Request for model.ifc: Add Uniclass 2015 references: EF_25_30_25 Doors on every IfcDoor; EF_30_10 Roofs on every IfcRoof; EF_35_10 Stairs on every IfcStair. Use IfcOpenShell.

First a look at what the model holds.

```python
import ifcopenshell

model = ifcopenshell.open("model.ifc")
print(model.schema)
print("classifications:", [c.Name for c in model.by_type("IfcClassification")])
for ifc_class in ("IfcDoor", "IfcRoof", "IfcStair", "IfcWall", "IfcWindow"):
    print(ifc_class, len(model.by_type(ifc_class)))
```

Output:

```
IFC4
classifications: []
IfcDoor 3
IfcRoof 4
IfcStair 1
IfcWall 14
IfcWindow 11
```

```python
import ifcopenshell
import ifcopenshell.api.classification

model = ifcopenshell.open("model.ifc")

system = ifcopenshell.api.classification.add_classification(model, classification="Uniclass 2015")

codes = {
    "IfcDoor": ("EF_25_30_25", "Doors"),
    "IfcRoof": ("EF_30_10", "Roofs"),
    "IfcStair": ("EF_35_10", "Stairs"),
}
for ifc_class, (code, name) in codes.items():
    products = model.by_type(ifc_class)
    ifcopenshell.api.classification.add_reference(
        model, products=products, classification=system, identification=code, name=name
    )
    print(code, len(products))

model.write("model_updated.ifc")
```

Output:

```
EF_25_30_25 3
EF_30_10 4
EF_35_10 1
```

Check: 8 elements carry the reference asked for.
